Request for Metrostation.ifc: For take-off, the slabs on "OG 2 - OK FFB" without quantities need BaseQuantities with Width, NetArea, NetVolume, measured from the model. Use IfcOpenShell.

First a look at what the model holds.

```python
import ifcopenshell
import ifcopenshell.util.element
import ifcopenshell.util.unit

model = ifcopenshell.open("Metrostation.ifc")
print(model.schema)
for unit_type in ("LENGTHUNIT", "AREAUNIT", "VOLUMEUNIT"):
    print(unit_type, ifcopenshell.util.unit.calculate_unit_scale(model, unit_type))
storey = next(s for s in model.by_type("IfcBuildingStorey") if s.Name == "OG 2 - OK FFB")
slabs = [e for e in ifcopenshell.util.element.get_decomposition(storey) if e.is_a("IfcSlab")]
for e in sorted(slabs, key=lambda e: e.id()):
    print(e.id(), e.is_a(), e.Name, list(ifcopenshell.util.element.get_psets(e, qtos_only=True)), sep=" | ")
```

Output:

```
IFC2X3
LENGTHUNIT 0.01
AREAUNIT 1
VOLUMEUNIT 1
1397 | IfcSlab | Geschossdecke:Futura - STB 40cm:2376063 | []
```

```python
import ifcopenshell
import ifcopenshell.api.pset
import ifcopenshell.geom
import ifcopenshell.util.element
import ifcopenshell.util.shape
import ifcopenshell.util.unit

model = ifcopenshell.open("Metrostation.ifc")
unit_scale = ifcopenshell.util.unit.calculate_unit_scale(model)
area_scale = ifcopenshell.util.unit.calculate_unit_scale(model, "AREAUNIT")
volume_scale = ifcopenshell.util.unit.calculate_unit_scale(model, "VOLUMEUNIT")
settings = ifcopenshell.geom.settings()

storey = next(s for s in model.by_type("IfcBuildingStorey") if s.Name == "OG 2 - OK FFB")
slabs = [e for e in ifcopenshell.util.element.get_decomposition(storey) if e.is_a("IfcSlab")]

for e in sorted(slabs, key=lambda e: e.id()):
    if ifcopenshell.util.element.get_psets(e, qtos_only=True, should_inherit=False):
        continue
    # Geometry comes back in metres, in the element's own axes.
    shape = ifcopenshell.geom.create_shape(settings, e)
    values = {
        "Width": ifcopenshell.util.shape.get_z(shape.geometry) / unit_scale,
        "NetArea": ifcopenshell.util.shape.get_footprint_area(shape.geometry) / area_scale,
        "NetVolume": ifcopenshell.util.shape.get_volume(shape.geometry) / volume_scale,
    }
    qto = ifcopenshell.api.pset.add_qto(model, product=e, name="BaseQuantities")
    ifcopenshell.api.pset.edit_qto(model, qto=qto, properties=values)
    print(e.id(), {k: round(v, 3) for k, v in values.items()})

model.write("Metrostation_v2.ifc")
```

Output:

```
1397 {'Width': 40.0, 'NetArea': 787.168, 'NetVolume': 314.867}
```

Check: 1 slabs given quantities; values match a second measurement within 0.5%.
